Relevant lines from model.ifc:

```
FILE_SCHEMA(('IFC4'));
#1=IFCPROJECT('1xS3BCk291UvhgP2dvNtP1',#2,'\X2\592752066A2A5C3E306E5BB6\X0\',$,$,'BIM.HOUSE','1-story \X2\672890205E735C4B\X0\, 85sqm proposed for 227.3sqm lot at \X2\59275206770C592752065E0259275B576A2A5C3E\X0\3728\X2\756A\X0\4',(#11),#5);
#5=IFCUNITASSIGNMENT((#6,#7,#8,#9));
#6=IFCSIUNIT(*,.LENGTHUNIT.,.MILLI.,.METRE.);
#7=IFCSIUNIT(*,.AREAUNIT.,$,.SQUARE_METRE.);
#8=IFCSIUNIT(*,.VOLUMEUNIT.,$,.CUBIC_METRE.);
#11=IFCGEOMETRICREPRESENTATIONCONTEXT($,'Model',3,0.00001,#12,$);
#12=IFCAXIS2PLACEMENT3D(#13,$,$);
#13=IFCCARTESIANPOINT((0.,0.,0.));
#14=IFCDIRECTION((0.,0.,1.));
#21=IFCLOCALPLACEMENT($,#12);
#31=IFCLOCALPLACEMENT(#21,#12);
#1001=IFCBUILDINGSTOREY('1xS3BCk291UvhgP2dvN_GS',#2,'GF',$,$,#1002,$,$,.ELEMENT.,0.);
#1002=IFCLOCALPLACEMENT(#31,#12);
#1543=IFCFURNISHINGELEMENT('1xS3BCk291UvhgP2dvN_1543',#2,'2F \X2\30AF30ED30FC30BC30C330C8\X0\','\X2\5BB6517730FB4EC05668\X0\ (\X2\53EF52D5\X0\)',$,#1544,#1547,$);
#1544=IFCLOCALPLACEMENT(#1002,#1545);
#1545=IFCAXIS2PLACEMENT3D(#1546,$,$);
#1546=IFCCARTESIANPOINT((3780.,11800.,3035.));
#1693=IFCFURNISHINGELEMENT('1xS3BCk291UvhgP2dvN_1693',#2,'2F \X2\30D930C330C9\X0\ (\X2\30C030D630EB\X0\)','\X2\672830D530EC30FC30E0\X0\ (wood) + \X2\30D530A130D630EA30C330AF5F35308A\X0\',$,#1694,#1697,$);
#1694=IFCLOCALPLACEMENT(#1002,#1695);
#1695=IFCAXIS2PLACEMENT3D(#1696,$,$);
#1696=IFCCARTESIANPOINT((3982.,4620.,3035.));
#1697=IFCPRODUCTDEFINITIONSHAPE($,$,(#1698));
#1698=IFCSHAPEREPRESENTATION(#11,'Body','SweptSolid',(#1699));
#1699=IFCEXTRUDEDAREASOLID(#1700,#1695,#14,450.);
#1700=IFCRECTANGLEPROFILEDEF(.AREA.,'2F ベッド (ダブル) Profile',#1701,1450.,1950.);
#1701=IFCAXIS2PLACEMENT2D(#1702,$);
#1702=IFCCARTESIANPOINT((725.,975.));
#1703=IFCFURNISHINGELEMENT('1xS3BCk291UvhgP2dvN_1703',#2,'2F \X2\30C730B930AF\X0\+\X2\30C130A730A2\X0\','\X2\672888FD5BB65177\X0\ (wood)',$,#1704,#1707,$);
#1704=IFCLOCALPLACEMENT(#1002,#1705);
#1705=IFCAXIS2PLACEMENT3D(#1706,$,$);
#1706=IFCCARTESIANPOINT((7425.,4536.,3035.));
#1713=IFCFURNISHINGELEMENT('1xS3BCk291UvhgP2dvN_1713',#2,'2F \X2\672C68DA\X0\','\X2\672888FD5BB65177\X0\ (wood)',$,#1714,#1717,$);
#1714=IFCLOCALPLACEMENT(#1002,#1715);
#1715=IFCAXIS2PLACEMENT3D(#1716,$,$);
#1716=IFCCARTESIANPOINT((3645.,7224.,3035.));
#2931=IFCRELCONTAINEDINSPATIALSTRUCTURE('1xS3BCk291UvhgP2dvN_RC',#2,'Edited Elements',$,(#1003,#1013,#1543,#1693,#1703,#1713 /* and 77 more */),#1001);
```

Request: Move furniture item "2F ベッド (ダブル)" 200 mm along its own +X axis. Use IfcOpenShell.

```python
import ifcopenshell
import ifcopenshell.api.geometry
import ifcopenshell.util.placement

model = ifcopenshell.open("model.ifc")

item = model.by_guid("1xS3BCk291UvhgP2dvN_1693")
matrix = ifcopenshell.util.placement.get_local_placement(item.ObjectPlacement)
matrix[:3, 3] += matrix[:3, 0] * 200.0
ifcopenshell.api.geometry.edit_object_placement(model, product=item, matrix=matrix, is_si=False)

print(ifcopenshell.util.placement.get_local_placement(item.ObjectPlacement).round(3) + 0.0)

model.write("model_rev.ifc")
```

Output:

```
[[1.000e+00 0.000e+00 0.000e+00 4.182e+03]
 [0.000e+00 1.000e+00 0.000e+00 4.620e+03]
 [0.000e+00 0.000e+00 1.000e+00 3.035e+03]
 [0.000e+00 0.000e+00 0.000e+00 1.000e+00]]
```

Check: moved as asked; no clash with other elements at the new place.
